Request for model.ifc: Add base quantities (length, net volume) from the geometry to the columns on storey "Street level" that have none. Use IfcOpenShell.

First a look at what the model holds.

```python
import ifcopenshell
import ifcopenshell.util.element
import ifcopenshell.util.unit

model = ifcopenshell.open("model.ifc")
print(model.schema)
for unit_type in ("LENGTHUNIT", "AREAUNIT", "VOLUMEUNIT"):
    print(unit_type, ifcopenshell.util.unit.calculate_unit_scale(model, unit_type))
storey = next(s for s in model.by_type("IfcBuildingStorey") if s.Name == "Street level")
columns = [e for e in ifcopenshell.util.element.get_decomposition(storey) if e.is_a("IfcColumn")]
for e in sorted(columns, key=lambda e: e.id()):
    print(e.id(), e.is_a(), e.Name, list(ifcopenshell.util.element.get_psets(e, qtos_only=True)), sep=" | ")
```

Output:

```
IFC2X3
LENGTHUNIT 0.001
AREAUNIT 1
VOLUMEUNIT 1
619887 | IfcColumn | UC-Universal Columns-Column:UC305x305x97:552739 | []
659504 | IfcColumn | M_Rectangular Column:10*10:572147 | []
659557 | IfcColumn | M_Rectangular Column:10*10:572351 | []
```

```python
import ifcopenshell
import ifcopenshell.api.pset
import ifcopenshell.geom
import ifcopenshell.util.element
import ifcopenshell.util.shape
import ifcopenshell.util.unit

model = ifcopenshell.open("model.ifc")
unit_scale = ifcopenshell.util.unit.calculate_unit_scale(model)
volume_scale = ifcopenshell.util.unit.calculate_unit_scale(model, "VOLUMEUNIT")
settings = ifcopenshell.geom.settings()

storey = next(s for s in model.by_type("IfcBuildingStorey") if s.Name == "Street level")
columns = [e for e in ifcopenshell.util.element.get_decomposition(storey) if e.is_a("IfcColumn")]

for e in sorted(columns, key=lambda e: e.id()):
    if ifcopenshell.util.element.get_psets(e, qtos_only=True, should_inherit=False):
        continue
    # Geometry comes back in metres, in the element's own axes.
    shape = ifcopenshell.geom.create_shape(settings, e)
    values = {
        "Length": ifcopenshell.util.shape.get_z(shape.geometry) / unit_scale,
        "NetVolume": ifcopenshell.util.shape.get_volume(shape.geometry) / volume_scale,
    }
    qto = ifcopenshell.api.pset.add_qto(model, product=e, name="BaseQuantities")
    ifcopenshell.api.pset.edit_qto(model, qto=qto, properties=values)
    print(e.id(), {k: round(v, 3) for k, v in values.items()})

model.write("model_v2.ifc")
```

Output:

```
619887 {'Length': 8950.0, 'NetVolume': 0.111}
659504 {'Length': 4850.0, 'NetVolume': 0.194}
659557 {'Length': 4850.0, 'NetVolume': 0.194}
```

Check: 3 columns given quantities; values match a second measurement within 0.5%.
